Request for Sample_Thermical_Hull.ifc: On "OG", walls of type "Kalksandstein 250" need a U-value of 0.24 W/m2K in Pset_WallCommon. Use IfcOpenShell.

First a look at what the model holds.

```python
import ifcopenshell
import ifcopenshell.util.element

model = ifcopenshell.open("Sample_Thermical_Hull.ifc")
print(model.schema)
storey = next(s for s in model.by_type("IfcBuildingStorey") if s.Name == "OG")
walls = [e for e in ifcopenshell.util.element.get_decomposition(storey) if e.is_a("IfcWall")]
seen = {}
for e in walls:
    element_type = ifcopenshell.util.element.get_type(e)
    key = (element_type.Name if element_type != e and element_type else None, ifcopenshell.util.element.get_pset(e, "Pset_WallCommon", "ThermalTransmittance"))
    seen[key] = seen.get(key, 0) + 1
for (name, value), count in sorted(seen.items(), key=str):
    print(count, "x", name, "|", value)
```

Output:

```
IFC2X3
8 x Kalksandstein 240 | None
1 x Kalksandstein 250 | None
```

```python
import ifcopenshell
import ifcopenshell.api.pset
import ifcopenshell.util.element

model = ifcopenshell.open("Sample_Thermical_Hull.ifc")

storey = next(s for s in model.by_type("IfcBuildingStorey") if s.Name == "OG")
walls = [e for e in ifcopenshell.util.element.get_decomposition(storey) if e.is_a("IfcWall")]

count = 0
for e in walls:
    element_type = ifcopenshell.util.element.get_type(e)
    if element_type in (None, e) or element_type.Name != "Kalksandstein 250":
        continue
    # add_pset returns the element's existing set when there is one.
    pset = ifcopenshell.api.pset.add_pset(model, product=e, name="Pset_WallCommon")
    ifcopenshell.api.pset.edit_pset(model, pset=pset, properties={"ThermalTransmittance": 0.24})
    count += 1

print(count, "walls updated")

model.write("Sample_Thermical_Hull_v2.ifc")
```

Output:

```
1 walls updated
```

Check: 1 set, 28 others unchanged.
